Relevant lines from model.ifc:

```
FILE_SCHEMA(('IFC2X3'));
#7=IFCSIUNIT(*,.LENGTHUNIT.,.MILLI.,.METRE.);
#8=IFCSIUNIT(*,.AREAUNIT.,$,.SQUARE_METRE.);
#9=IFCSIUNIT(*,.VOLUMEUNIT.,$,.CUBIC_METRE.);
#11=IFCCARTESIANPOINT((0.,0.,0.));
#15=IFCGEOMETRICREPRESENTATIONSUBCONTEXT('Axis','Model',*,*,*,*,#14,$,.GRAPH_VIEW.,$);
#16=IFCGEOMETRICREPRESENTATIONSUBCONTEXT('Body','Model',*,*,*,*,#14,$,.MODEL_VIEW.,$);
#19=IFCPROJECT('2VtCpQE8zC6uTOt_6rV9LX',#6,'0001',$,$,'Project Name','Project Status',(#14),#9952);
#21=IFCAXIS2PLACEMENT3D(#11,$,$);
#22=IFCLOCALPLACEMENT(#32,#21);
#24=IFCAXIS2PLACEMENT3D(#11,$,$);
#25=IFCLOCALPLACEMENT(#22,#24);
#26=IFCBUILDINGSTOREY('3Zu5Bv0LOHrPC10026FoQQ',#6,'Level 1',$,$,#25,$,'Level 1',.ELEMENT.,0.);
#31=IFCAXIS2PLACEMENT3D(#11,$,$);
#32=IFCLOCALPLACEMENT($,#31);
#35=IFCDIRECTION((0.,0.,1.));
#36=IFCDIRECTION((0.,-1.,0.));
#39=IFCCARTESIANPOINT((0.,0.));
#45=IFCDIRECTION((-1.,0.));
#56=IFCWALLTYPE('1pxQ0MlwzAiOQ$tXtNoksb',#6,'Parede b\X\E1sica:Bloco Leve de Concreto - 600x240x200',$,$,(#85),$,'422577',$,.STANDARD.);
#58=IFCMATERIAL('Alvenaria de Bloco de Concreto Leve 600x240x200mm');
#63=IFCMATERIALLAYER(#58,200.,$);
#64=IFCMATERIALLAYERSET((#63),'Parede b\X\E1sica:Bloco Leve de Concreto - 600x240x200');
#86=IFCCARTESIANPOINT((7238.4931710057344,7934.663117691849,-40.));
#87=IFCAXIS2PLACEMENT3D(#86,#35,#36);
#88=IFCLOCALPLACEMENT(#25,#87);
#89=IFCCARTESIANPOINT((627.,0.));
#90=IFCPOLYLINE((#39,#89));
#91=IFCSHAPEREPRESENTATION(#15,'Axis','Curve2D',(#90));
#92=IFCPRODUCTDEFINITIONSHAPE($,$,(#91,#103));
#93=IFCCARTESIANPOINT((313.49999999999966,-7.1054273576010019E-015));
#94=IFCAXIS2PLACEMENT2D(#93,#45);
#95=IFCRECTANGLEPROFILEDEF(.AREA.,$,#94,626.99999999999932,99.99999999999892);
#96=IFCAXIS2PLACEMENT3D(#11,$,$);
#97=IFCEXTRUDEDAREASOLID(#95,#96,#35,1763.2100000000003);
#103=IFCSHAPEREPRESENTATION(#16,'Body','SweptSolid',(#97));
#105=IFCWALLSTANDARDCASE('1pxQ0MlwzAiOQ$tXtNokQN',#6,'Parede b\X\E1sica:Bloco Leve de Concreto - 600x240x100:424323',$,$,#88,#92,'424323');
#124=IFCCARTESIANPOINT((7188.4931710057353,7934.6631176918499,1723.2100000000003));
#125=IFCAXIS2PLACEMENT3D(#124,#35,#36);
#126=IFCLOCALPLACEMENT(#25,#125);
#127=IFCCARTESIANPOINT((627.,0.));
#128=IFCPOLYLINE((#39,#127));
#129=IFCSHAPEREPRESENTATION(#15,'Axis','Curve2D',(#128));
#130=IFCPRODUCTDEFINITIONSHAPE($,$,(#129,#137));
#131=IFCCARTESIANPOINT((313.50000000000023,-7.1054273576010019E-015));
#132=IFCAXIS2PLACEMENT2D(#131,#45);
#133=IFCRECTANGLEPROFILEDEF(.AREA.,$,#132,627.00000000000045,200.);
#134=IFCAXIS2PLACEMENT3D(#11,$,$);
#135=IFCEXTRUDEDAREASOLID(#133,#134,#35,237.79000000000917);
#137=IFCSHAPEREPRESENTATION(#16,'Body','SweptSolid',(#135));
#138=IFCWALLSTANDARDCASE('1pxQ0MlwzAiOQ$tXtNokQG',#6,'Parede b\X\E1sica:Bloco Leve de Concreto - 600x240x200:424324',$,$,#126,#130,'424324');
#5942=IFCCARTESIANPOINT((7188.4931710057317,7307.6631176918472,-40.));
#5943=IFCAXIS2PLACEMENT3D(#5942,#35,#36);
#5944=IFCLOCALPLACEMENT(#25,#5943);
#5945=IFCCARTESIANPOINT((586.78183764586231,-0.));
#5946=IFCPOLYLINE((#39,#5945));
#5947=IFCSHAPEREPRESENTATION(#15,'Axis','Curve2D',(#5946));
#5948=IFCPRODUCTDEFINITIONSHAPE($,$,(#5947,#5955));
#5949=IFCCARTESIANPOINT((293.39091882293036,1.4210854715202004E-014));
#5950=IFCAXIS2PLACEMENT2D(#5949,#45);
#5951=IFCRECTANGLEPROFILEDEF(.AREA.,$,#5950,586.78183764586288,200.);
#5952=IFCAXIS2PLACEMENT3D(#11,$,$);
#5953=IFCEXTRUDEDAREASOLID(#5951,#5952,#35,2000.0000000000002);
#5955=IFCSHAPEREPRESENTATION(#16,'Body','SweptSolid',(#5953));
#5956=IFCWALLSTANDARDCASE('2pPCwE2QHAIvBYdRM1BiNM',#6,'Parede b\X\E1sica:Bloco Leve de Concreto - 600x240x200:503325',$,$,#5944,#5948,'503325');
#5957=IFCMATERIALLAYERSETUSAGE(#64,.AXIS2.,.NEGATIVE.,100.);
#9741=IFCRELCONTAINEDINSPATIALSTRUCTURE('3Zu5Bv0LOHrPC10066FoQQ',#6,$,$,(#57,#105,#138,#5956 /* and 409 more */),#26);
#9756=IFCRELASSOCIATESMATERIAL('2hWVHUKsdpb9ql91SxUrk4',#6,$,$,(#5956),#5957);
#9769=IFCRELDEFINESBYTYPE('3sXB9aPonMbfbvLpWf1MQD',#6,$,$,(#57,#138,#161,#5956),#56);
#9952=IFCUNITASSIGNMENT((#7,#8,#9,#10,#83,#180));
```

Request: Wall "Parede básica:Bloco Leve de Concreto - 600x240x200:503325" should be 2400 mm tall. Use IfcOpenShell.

```python
import ifcopenshell
import ifcopenshell.geom
import ifcopenshell.util.representation
import ifcopenshell.util.shape
import ifcopenshell.util.unit

model = ifcopenshell.open("model.ifc")
unit_scale = ifcopenshell.util.unit.calculate_unit_scale(model)
settings = ifcopenshell.geom.settings()


def volume(element):
    """Net volume in cubic metres, openings subtracted."""
    shape = ifcopenshell.geom.create_shape(settings, element)
    return ifcopenshell.util.shape.get_volume(shape.geometry)


wall = model.by_id(5956)
before = volume(wall)

body = ifcopenshell.util.representation.get_representation(wall, "Model", "Body")
solid = body.Items[0]
old_height = solid.Depth
solid.Depth = 2.4 / unit_scale
after = volume(wall)

print(f"height {old_height:g} -> {solid.Depth:g}, volume {before:.3f} -> {after:.3f} m3")

model.write("model_updated.ifc")
```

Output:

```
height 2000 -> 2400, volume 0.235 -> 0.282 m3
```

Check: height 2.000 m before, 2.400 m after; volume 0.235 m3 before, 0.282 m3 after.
